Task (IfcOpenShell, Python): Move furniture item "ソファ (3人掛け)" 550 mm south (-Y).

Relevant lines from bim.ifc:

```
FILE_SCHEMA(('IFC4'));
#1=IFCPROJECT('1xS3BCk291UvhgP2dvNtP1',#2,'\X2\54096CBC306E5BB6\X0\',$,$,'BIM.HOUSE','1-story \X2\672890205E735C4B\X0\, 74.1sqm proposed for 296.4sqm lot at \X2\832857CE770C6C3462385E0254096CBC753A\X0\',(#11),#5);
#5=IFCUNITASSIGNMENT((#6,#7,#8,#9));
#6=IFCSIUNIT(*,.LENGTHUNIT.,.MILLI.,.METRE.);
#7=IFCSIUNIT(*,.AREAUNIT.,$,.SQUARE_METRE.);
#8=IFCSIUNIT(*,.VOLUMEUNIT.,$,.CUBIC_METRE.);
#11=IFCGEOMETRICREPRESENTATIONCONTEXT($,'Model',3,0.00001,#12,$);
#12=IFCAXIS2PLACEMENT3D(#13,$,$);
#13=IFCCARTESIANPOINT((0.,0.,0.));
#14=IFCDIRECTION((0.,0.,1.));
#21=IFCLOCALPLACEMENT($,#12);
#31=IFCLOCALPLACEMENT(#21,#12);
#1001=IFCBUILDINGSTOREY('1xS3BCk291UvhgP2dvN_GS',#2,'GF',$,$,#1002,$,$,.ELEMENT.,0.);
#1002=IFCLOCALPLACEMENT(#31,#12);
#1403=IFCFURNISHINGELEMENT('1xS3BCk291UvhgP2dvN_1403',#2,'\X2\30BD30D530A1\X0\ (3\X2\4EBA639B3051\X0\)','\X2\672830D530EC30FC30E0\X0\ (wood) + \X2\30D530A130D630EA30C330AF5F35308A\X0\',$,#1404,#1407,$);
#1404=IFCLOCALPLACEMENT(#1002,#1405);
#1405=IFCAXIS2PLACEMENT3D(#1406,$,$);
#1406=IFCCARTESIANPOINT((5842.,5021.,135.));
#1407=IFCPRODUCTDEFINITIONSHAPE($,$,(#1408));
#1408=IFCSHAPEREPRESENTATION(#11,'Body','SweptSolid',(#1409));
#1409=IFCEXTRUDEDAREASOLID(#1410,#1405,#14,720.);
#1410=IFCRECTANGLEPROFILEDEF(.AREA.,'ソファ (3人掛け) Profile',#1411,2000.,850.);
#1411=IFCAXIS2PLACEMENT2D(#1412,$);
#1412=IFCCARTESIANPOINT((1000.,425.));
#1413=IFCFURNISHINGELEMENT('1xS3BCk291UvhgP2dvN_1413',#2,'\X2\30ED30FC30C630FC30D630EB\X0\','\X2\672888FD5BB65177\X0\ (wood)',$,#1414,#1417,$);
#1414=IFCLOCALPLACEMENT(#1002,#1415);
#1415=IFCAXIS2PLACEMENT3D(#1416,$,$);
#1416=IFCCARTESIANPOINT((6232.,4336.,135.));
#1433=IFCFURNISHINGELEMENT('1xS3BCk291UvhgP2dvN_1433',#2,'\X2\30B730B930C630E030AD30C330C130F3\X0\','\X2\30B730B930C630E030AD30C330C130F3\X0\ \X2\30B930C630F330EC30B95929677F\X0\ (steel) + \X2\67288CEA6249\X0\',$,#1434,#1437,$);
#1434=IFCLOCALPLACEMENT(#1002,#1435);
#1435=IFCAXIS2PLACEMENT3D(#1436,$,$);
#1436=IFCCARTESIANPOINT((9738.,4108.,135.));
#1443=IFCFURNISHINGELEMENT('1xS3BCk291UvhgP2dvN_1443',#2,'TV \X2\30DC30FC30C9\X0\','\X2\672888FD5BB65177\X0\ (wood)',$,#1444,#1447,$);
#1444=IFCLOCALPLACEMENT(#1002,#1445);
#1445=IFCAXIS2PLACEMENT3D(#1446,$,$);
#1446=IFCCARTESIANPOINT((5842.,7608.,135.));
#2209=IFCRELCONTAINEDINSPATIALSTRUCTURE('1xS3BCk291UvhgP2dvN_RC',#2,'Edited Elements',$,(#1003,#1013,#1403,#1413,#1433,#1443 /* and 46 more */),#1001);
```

```python
import ifcopenshell
import ifcopenshell.api.geometry
import ifcopenshell.util.placement
import ifcopenshell.util.unit

model = ifcopenshell.open("bim.ifc")
unit_scale = ifcopenshell.util.unit.calculate_unit_scale(model)

item = model.by_guid("1xS3BCk291UvhgP2dvN_1403")
matrix = ifcopenshell.util.placement.get_local_placement(item.ObjectPlacement)
matrix[1, 3] -= 0.55 / unit_scale
ifcopenshell.api.geometry.edit_object_placement(model, product=item, matrix=matrix, is_si=False)

print(ifcopenshell.util.placement.get_local_placement(item.ObjectPlacement).round(3) + 0.0)

model.write("bim_updated.ifc")
```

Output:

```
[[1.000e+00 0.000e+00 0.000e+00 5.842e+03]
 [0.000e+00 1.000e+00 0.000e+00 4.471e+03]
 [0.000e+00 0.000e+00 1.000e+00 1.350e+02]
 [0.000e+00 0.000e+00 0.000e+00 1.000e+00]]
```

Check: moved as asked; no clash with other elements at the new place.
